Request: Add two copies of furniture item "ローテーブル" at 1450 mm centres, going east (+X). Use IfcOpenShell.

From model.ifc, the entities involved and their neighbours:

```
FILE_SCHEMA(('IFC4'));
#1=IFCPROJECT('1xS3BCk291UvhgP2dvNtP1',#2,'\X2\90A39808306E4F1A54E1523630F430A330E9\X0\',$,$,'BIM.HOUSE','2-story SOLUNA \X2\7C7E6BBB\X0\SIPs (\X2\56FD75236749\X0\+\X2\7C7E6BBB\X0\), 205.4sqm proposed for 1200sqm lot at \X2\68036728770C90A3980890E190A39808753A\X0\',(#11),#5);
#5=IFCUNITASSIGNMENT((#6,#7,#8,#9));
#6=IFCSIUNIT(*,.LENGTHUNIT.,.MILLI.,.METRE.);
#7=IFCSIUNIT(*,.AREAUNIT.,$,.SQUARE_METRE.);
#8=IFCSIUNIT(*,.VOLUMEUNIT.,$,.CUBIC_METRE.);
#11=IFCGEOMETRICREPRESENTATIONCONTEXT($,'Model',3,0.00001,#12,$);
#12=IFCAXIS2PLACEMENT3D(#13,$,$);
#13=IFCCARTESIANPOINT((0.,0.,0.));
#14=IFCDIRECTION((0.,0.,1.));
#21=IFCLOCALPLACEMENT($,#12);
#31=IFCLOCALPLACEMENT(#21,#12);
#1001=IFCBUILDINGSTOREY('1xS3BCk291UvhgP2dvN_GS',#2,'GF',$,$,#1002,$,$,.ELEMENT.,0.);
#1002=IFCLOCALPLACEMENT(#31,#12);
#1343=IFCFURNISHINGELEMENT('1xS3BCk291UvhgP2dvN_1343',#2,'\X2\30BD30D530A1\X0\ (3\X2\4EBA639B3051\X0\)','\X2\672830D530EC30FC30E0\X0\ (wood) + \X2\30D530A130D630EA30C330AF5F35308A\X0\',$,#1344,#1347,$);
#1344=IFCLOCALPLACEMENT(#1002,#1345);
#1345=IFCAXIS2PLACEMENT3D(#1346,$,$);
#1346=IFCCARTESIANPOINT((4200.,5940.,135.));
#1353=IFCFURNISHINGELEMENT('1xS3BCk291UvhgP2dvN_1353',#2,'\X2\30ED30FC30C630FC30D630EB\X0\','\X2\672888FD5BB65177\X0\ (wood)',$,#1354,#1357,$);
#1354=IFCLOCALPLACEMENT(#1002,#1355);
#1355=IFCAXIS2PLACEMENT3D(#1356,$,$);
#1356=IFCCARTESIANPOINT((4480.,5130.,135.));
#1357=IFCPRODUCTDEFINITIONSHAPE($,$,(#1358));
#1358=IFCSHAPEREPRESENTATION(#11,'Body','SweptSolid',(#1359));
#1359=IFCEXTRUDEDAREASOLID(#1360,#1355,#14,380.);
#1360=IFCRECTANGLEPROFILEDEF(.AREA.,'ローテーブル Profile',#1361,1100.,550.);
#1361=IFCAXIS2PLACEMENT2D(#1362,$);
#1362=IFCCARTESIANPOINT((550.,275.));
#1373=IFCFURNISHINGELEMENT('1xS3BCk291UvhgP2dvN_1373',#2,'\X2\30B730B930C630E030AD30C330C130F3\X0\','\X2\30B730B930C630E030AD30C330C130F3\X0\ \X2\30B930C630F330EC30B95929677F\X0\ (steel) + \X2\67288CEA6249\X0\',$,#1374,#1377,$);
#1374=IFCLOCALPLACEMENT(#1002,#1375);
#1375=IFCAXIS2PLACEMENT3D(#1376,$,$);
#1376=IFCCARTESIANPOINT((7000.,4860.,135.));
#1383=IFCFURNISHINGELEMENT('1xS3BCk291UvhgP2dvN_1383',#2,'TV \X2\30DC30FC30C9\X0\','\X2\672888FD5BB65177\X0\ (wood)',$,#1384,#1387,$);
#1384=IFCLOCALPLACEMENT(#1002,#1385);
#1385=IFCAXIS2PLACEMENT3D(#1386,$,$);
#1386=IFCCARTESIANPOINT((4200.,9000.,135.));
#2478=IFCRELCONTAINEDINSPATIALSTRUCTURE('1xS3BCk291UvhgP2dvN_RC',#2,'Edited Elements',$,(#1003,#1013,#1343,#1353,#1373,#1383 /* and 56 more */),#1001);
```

```python
import numpy as np
import ifcopenshell
import ifcopenshell.api.geometry
import ifcopenshell.api.root
import ifcopenshell.util.element
import ifcopenshell.util.placement
import ifcopenshell.util.unit

model = ifcopenshell.open("model.ifc")
unit_scale = ifcopenshell.util.unit.calculate_unit_scale(model)


def reuse_history(source, copy):
    """copy_class also copies each property set's owner history, people and application; keep the originals."""
    for rel in copy.IsDefinedBy:
        if rel.is_a("IfcRelDefinesByProperties") and (history := rel.RelatingPropertyDefinition.OwnerHistory):
            rel.RelatingPropertyDefinition.OwnerHistory = source.OwnerHistory
            ifcopenshell.util.element.remove_deep2(model, history)


source = model.by_guid("1xS3BCk291UvhgP2dvN_1353")
base = ifcopenshell.util.placement.get_local_placement(source.ObjectPlacement)
step = np.array([1.0, 0.0, 0.0]) * 1.45 / unit_scale

for i in range(1, 3):
    copy = ifcopenshell.api.root.copy_class(model, product=source)
    copy.Representation = ifcopenshell.util.element.copy_deep(
        model, source.Representation, exclude=["IfcGeometricRepresentationContext", "IfcRepresentationMap"]
    )
    reuse_history(source, copy)
    matrix = base.copy()
    matrix[:3, 3] += i * step
    print("added at", matrix[:3, 3].round(3) + 0.0)
    ifcopenshell.api.geometry.edit_object_placement(model, product=copy, matrix=matrix, is_si=False)

model.write("model_edited.ifc")
```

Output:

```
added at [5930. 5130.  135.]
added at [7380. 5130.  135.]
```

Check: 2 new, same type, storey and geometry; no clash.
